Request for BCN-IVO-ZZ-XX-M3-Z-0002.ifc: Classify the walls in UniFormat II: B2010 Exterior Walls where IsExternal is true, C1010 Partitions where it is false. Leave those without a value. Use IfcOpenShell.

First a look at what the model holds.

```python
import ifcopenshell
import ifcopenshell.util.element

model = ifcopenshell.open("BCN-IVO-ZZ-XX-M3-Z-0002.ifc")
print(model.schema)
print("classifications:", [c.Name for c in model.by_type("IfcClassification")])
values = [ifcopenshell.util.element.get_pset(e, "Pset_WallCommon", "IsExternal") for e in model.by_type("IfcWall")]
for value in (True, False, None):
    print("IsExternal", value, values.count(value))
```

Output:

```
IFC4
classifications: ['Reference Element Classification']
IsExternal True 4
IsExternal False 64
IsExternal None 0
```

```python
import ifcopenshell
import ifcopenshell.api.classification
import ifcopenshell.util.element

model = ifcopenshell.open("BCN-IVO-ZZ-XX-M3-Z-0002.ifc")

system = ifcopenshell.api.classification.add_classification(model, classification="UniFormat II")

walls = model.by_type("IfcWall")
external = {e: ifcopenshell.util.element.get_pset(e, "Pset_WallCommon", "IsExternal") for e in walls}
for flag, code, name in ((True, "B2010", "Exterior Walls"), (False, "C1010", "Partitions")):
    products = [e for e in walls if external[e] is flag]
    ifcopenshell.api.classification.add_reference(
        model, products=products, classification=system, identification=code, name=name
    )
    print(code, len(products))

model.write("BCN-IVO-ZZ-XX-M3-Z-0002_rev.ifc")
```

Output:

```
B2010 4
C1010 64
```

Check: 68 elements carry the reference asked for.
